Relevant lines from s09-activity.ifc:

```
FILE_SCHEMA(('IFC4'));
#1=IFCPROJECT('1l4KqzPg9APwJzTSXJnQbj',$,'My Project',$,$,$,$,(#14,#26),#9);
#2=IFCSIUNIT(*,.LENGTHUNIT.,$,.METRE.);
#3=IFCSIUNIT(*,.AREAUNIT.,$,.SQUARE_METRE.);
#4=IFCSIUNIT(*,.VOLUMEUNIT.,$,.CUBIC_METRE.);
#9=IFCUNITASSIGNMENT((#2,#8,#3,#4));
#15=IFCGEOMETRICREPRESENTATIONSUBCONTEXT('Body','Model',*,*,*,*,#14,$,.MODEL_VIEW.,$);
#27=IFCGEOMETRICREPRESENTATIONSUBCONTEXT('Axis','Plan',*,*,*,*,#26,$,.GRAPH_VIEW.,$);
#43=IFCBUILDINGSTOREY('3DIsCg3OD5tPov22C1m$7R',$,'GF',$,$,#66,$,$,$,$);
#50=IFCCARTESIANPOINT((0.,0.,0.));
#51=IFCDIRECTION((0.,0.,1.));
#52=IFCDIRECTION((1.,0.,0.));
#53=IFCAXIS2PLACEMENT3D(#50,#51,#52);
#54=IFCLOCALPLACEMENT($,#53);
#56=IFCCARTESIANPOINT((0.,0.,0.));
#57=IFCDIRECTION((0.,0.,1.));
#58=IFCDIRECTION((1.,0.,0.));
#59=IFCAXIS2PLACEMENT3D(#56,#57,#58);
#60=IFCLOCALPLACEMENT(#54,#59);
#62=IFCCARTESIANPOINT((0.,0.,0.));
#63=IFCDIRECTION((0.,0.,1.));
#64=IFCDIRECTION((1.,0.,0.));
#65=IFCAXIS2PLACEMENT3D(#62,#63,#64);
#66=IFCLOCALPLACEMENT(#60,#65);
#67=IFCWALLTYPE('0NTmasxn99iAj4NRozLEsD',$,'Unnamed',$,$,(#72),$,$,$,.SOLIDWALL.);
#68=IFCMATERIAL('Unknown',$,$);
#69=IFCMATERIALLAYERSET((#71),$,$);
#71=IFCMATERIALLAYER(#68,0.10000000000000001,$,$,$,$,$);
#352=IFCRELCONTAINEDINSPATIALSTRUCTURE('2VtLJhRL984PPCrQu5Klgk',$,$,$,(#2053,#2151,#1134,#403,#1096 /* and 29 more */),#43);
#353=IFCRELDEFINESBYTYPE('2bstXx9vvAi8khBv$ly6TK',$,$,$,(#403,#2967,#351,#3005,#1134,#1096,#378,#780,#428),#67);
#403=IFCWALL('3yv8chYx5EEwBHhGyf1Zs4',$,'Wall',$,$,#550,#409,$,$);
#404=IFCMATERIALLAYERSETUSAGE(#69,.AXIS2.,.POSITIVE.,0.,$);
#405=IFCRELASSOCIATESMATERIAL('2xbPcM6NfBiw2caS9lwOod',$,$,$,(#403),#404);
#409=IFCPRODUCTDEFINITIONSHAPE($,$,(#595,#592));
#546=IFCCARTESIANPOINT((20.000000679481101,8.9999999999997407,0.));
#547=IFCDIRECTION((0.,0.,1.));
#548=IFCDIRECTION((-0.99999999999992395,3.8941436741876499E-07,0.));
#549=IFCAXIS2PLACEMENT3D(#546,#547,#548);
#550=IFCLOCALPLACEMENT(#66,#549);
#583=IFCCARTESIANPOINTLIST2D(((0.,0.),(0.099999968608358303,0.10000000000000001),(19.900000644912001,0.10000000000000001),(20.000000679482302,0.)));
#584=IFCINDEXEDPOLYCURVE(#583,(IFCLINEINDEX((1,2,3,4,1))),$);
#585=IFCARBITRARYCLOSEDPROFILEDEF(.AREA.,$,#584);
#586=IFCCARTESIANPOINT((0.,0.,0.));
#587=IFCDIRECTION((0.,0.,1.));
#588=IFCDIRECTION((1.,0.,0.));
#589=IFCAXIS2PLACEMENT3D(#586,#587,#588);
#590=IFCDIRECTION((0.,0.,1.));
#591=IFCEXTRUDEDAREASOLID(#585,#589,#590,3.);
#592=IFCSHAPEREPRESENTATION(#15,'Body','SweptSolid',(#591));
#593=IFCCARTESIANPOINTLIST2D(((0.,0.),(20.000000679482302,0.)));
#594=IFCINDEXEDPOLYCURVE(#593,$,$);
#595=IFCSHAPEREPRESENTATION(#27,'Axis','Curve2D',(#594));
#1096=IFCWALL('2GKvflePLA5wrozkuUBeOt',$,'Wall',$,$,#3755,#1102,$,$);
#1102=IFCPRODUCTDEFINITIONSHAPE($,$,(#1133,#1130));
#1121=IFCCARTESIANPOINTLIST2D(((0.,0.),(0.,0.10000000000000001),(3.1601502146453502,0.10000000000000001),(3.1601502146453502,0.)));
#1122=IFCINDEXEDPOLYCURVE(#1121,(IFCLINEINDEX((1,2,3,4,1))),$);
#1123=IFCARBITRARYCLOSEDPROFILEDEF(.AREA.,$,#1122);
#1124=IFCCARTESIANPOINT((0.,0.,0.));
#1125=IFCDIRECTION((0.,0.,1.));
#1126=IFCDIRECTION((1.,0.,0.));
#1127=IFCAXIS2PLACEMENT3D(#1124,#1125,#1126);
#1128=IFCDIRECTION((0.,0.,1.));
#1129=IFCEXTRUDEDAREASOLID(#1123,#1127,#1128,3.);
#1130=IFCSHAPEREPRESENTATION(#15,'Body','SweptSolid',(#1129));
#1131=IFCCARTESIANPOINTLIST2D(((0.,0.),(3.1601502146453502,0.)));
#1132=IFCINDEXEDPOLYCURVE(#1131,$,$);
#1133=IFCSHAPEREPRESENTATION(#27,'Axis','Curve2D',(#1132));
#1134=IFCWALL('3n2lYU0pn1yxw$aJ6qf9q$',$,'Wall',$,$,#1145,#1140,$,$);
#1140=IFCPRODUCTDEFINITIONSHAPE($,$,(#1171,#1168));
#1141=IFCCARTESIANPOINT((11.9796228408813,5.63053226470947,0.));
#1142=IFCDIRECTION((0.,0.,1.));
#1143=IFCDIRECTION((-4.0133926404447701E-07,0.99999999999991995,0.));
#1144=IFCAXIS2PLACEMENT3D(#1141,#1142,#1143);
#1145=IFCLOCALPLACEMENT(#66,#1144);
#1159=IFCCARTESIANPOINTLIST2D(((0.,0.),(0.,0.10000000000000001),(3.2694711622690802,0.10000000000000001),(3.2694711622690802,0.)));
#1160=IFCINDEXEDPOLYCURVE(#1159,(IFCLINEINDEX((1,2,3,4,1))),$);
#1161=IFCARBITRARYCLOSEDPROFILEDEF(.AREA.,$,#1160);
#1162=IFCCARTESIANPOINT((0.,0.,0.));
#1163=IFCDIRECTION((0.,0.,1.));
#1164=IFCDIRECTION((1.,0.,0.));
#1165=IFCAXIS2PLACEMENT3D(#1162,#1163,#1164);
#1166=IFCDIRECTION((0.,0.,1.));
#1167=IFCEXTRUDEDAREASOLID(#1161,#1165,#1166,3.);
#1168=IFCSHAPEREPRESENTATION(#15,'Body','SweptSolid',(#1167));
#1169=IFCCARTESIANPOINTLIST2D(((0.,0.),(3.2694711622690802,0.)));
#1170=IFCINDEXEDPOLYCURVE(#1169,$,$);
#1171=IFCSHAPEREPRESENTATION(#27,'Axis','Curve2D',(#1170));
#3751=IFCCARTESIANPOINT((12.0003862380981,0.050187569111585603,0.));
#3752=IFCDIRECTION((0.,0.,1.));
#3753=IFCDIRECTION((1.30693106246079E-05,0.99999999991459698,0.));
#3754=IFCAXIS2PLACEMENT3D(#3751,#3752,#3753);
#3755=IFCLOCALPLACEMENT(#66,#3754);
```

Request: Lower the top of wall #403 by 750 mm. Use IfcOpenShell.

```python
import ifcopenshell
import ifcopenshell.geom
import ifcopenshell.util.representation
import ifcopenshell.util.shape
import ifcopenshell.util.unit

model = ifcopenshell.open("s09-activity.ifc")
unit_scale = ifcopenshell.util.unit.calculate_unit_scale(model)
settings = ifcopenshell.geom.settings()


def volume(element):
    """Net volume in cubic metres, openings subtracted."""
    shape = ifcopenshell.geom.create_shape(settings, element)
    return ifcopenshell.util.shape.get_volume(shape.geometry)


wall = model.by_guid("3yv8chYx5EEwBHhGyf1Zs4")
before = volume(wall)

body = ifcopenshell.util.representation.get_representation(wall, "Model", "Body")
solid = body.Items[0]
old_height = solid.Depth
solid.Depth -= 0.75 / unit_scale
after = volume(wall)

print(f"height {old_height:g} -> {solid.Depth:g}, volume {before:.3f} -> {after:.3f} m3")

model.write("s09-activity_v2.ifc")
```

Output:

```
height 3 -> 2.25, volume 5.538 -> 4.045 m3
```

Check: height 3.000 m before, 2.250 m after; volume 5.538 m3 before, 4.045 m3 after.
